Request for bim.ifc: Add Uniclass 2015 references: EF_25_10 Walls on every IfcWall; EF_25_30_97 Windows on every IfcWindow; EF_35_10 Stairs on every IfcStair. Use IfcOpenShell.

First a look at what the model holds.

```python
import ifcopenshell

model = ifcopenshell.open("bim.ifc")
print(model.schema)
print("classifications:", [c.Name for c in model.by_type("IfcClassification")])
for ifc_class in ("IfcDoor", "IfcRoof", "IfcStair", "IfcWall", "IfcWindow"):
    print(ifc_class, len(model.by_type(ifc_class)))
```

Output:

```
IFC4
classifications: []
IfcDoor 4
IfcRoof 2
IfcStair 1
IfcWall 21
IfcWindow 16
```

```python
import ifcopenshell
import ifcopenshell.api.classification

model = ifcopenshell.open("bim.ifc")

system = ifcopenshell.api.classification.add_classification(model, classification="Uniclass 2015")

codes = {
    "IfcWall": ("EF_25_10", "Walls"),
    "IfcWindow": ("EF_25_30_97", "Windows"),
    "IfcStair": ("EF_35_10", "Stairs"),
}
for ifc_class, (code, name) in codes.items():
    products = model.by_type(ifc_class)
    ifcopenshell.api.classification.add_reference(
        model, products=products, classification=system, identification=code, name=name
    )
    print(code, len(products))

model.write("bim_updated.ifc")
```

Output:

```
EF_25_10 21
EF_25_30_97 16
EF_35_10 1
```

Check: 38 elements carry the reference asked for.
